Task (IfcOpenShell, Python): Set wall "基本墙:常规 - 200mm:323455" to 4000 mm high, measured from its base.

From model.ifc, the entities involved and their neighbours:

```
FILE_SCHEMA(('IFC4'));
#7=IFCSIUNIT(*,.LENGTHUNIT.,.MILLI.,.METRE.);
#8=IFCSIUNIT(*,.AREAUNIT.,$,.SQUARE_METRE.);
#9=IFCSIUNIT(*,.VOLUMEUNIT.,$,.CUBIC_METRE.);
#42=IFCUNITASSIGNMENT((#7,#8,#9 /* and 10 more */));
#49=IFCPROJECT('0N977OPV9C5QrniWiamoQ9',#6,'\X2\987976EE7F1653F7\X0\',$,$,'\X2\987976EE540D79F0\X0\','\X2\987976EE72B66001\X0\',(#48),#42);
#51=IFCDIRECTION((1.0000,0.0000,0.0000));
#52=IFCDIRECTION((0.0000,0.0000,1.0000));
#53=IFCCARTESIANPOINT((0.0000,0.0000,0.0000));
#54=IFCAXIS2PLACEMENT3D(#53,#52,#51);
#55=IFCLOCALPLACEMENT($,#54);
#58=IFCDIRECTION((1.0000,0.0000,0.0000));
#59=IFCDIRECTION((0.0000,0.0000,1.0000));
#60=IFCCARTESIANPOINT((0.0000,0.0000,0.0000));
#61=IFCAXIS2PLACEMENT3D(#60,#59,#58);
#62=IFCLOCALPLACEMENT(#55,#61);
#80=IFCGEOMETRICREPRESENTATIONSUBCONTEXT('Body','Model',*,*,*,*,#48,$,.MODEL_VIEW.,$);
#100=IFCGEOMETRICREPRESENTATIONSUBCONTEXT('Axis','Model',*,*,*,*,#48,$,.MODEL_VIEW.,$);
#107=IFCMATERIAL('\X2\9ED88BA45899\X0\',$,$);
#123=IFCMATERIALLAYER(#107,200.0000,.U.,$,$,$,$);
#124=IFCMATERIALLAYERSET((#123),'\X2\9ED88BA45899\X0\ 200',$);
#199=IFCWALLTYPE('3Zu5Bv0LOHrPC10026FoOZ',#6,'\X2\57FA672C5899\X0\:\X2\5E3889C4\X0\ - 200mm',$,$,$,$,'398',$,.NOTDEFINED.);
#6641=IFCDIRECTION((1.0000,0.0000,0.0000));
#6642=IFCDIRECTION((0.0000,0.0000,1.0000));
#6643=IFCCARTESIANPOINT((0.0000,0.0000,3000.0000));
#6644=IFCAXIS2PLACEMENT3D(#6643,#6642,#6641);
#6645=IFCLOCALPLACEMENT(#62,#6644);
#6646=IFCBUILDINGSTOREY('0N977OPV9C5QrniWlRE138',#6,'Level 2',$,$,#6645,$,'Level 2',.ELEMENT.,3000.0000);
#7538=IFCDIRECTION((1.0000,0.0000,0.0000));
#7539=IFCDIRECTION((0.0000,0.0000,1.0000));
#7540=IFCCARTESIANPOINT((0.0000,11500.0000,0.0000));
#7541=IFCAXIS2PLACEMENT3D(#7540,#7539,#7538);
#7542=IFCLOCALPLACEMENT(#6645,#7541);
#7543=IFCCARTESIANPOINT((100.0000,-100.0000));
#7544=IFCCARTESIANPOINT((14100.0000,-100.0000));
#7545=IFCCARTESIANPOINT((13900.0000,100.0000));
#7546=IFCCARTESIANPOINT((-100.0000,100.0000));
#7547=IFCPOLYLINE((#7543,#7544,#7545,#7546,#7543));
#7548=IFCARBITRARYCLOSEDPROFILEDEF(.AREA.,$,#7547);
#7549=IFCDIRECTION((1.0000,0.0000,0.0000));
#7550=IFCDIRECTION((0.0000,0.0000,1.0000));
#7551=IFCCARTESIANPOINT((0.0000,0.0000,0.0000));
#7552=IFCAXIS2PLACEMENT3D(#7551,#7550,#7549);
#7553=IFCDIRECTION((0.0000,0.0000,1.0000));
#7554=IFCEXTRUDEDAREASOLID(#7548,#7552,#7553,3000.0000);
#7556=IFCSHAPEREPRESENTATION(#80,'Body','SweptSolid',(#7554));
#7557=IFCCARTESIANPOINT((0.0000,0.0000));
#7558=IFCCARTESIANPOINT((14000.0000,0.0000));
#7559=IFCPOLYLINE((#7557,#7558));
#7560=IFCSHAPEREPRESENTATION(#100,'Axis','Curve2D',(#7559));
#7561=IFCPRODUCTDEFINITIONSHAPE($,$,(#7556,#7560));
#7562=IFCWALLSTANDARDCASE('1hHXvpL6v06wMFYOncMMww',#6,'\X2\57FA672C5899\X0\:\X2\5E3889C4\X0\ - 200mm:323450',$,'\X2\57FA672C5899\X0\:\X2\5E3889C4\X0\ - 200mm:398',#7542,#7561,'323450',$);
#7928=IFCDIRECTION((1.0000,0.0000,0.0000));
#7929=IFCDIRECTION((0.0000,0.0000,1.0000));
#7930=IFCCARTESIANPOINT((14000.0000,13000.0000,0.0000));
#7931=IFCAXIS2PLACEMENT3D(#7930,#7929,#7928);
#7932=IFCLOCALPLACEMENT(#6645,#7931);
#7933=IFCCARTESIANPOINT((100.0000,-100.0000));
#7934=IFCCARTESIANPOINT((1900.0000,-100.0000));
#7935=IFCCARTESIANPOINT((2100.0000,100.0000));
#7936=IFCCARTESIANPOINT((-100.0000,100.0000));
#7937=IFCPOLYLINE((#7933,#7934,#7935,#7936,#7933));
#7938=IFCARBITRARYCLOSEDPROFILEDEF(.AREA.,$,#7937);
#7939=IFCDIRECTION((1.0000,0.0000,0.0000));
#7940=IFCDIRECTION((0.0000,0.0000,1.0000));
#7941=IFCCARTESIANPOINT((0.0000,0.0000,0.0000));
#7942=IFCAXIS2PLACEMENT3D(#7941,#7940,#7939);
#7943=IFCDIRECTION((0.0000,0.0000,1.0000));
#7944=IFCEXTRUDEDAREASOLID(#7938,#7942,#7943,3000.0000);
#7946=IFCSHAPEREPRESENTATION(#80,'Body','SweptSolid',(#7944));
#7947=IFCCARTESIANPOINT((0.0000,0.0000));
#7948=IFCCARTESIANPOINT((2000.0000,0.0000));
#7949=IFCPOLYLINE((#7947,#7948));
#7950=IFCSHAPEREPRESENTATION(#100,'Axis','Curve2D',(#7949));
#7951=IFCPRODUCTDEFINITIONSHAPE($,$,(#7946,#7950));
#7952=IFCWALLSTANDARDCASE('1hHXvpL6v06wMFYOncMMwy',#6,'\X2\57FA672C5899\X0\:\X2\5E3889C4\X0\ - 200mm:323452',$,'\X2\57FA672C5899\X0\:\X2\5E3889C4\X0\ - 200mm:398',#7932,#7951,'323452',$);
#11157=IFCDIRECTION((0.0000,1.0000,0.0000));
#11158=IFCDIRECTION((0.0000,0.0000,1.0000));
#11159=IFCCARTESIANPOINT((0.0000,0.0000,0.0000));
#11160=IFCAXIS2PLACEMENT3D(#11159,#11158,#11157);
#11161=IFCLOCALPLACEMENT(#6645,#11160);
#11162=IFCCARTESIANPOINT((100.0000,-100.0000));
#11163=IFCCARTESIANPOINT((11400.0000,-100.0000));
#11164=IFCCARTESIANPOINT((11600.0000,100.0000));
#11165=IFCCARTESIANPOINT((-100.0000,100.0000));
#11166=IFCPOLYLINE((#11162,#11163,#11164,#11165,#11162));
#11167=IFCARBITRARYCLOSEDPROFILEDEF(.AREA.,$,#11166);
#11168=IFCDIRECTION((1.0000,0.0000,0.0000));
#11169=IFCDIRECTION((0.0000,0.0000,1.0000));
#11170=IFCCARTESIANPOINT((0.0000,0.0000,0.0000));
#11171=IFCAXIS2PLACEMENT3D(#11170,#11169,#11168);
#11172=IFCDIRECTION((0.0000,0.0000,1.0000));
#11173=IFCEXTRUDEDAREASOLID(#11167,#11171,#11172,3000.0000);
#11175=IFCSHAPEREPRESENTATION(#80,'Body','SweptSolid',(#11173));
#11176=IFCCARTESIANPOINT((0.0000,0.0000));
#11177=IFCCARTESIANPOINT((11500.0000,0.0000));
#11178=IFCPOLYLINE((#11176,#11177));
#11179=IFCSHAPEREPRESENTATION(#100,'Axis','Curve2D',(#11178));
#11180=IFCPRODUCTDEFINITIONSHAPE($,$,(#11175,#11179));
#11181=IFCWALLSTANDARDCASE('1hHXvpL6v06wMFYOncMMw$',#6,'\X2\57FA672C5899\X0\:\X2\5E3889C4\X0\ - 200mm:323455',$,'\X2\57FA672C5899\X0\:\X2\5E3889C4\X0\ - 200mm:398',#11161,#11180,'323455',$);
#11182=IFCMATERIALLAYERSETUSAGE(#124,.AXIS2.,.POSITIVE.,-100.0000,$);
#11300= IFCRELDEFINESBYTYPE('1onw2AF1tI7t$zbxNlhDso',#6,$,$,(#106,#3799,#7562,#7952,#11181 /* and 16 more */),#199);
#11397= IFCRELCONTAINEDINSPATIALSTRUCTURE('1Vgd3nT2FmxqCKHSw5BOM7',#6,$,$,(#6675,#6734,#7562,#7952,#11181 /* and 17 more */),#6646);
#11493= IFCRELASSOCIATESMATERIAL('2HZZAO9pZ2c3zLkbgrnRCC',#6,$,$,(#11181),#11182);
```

```python
import ifcopenshell
import ifcopenshell.geom
import ifcopenshell.util.representation
import ifcopenshell.util.shape

model = ifcopenshell.open("model.ifc")
settings = ifcopenshell.geom.settings()


def volume(element):
    """Net volume in cubic metres, openings subtracted."""
    shape = ifcopenshell.geom.create_shape(settings, element)
    return ifcopenshell.util.shape.get_volume(shape.geometry)


wall = model.by_guid("1hHXvpL6v06wMFYOncMMw$")
before = volume(wall)

body = ifcopenshell.util.representation.get_representation(wall, "Model", "Body")
solid = body.Items[0]
old_height = solid.Depth
solid.Depth = 4000.0
after = volume(wall)

print(f"height {old_height:g} -> {solid.Depth:g}, volume {before:.3f} -> {after:.3f} m3")

model.write("model_updated.ifc")
```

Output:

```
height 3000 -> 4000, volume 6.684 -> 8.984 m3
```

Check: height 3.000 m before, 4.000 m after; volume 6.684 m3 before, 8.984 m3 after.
